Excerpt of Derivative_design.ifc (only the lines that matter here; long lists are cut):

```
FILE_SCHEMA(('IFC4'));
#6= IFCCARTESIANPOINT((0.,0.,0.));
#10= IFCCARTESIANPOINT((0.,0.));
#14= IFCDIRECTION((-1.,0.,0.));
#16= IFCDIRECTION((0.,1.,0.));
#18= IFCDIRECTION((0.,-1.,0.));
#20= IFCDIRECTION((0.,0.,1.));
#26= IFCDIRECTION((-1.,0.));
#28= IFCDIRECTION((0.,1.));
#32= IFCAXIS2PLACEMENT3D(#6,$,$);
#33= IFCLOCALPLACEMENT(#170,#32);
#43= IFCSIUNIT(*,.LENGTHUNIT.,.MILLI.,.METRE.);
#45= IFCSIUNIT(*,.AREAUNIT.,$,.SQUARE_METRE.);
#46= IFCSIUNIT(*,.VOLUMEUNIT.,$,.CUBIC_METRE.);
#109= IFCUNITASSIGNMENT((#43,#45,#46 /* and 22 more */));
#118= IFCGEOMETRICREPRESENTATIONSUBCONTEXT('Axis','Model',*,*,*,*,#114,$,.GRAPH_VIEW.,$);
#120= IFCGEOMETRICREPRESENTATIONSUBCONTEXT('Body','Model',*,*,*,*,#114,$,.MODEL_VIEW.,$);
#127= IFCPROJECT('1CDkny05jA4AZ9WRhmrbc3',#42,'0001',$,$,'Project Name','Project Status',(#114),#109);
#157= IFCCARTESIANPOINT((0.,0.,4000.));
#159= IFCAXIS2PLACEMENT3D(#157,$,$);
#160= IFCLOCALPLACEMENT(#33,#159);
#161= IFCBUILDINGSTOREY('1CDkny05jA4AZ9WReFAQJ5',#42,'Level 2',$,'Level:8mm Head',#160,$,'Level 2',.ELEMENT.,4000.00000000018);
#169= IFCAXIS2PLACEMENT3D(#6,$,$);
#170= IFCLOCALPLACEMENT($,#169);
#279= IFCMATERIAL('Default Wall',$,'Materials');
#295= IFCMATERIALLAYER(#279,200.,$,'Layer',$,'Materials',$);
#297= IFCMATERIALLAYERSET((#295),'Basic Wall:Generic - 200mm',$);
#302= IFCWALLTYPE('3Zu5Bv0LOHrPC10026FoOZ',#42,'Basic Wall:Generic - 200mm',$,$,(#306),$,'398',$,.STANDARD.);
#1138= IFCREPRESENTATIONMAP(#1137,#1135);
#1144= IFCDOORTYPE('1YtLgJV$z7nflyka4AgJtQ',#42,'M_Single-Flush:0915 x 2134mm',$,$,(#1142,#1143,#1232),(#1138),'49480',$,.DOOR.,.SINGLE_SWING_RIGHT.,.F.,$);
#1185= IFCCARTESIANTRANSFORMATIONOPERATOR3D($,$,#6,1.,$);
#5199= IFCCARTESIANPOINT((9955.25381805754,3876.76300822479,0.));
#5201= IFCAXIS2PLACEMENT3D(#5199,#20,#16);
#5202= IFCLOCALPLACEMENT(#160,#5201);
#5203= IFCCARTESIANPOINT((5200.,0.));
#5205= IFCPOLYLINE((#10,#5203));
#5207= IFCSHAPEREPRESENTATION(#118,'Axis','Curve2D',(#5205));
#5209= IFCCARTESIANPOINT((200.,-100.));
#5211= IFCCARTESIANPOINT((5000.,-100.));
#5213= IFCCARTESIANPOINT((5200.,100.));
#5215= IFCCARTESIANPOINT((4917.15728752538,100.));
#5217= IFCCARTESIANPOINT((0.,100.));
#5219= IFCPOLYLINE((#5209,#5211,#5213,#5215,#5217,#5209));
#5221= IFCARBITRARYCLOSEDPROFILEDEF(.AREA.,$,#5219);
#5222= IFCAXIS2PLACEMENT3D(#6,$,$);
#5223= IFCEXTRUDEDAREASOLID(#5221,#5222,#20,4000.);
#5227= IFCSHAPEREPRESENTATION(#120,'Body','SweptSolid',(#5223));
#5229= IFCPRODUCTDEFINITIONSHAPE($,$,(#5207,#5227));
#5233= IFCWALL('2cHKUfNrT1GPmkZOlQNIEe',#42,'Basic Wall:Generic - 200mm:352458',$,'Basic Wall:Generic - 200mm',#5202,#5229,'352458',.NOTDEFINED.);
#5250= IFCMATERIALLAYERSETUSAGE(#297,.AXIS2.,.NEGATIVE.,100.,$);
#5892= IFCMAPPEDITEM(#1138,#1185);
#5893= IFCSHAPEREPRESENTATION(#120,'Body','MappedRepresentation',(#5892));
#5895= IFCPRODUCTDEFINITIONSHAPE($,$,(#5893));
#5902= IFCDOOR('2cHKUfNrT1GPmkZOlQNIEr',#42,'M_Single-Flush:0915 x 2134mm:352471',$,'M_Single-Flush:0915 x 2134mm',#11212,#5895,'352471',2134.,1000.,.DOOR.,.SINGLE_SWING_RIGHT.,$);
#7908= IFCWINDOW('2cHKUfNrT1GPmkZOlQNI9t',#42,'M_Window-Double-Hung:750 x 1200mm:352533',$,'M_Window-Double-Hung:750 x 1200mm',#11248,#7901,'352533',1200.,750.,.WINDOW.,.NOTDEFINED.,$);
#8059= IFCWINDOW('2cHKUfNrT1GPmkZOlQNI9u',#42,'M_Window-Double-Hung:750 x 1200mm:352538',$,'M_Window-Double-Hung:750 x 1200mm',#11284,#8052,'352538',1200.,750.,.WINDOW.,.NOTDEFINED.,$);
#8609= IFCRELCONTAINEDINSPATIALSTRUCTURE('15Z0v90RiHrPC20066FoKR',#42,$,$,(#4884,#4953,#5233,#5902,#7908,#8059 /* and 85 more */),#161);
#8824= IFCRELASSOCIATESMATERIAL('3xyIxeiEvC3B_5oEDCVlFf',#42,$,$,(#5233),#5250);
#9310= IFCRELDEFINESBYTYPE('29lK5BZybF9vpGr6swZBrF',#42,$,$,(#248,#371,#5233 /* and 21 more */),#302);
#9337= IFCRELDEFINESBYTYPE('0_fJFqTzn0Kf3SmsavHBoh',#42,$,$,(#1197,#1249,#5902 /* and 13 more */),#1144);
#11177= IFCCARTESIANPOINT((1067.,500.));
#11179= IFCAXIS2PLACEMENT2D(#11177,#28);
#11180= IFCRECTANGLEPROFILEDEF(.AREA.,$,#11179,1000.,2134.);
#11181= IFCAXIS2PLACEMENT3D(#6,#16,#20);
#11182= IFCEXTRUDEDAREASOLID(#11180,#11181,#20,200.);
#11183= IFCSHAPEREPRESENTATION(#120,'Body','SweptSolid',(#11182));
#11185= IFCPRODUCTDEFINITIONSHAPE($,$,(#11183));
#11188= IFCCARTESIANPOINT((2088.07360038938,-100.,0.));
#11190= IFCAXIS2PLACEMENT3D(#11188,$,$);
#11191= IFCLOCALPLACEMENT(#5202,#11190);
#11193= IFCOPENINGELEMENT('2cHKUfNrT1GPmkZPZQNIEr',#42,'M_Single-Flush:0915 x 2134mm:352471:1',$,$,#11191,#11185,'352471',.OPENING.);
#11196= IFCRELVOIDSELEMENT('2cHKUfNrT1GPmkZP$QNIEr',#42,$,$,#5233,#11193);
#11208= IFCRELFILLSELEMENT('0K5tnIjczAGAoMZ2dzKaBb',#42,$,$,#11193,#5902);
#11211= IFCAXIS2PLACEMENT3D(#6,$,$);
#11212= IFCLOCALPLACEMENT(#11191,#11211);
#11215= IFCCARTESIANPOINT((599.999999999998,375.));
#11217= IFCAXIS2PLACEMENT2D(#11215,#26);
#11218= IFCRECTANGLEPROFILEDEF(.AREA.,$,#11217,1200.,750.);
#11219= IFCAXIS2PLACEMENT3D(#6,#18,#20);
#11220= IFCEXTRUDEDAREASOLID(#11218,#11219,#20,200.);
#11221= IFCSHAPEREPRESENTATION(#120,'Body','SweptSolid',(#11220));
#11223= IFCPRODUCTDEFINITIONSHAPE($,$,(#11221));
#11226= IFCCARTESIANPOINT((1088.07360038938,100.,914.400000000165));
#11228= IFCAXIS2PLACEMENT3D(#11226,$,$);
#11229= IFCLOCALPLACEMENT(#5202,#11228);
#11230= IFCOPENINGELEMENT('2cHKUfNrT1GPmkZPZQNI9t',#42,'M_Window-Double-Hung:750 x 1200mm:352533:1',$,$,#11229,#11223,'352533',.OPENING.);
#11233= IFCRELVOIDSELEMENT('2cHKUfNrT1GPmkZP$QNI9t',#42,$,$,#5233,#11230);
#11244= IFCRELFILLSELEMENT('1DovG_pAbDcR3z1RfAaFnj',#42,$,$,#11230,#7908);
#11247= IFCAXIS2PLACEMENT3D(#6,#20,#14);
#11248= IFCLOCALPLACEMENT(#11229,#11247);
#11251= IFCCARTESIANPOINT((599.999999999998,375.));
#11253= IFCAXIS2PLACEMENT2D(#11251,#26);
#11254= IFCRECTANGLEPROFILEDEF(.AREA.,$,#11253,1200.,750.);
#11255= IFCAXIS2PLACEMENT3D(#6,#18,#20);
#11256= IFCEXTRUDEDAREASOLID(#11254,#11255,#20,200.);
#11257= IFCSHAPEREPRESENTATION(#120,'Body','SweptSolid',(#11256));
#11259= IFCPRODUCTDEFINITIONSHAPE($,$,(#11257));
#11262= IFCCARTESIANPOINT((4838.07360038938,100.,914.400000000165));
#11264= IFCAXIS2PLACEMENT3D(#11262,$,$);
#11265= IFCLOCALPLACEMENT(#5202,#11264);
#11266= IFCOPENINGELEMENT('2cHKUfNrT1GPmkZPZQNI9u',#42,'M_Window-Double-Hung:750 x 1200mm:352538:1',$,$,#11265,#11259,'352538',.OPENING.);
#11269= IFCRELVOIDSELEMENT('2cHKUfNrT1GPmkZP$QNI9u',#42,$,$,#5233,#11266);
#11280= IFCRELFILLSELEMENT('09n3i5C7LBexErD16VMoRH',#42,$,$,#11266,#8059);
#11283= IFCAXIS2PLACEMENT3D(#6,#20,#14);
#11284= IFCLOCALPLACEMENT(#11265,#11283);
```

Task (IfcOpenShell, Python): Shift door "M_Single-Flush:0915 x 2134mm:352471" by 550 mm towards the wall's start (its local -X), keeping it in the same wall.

```python
import ifcopenshell
import ifcopenshell.api.geometry
import ifcopenshell.util.placement

model = ifcopenshell.open("Derivative_design.ifc")

door = model.by_id(5902)
opening = door.FillsVoids[0].RelatingOpeningElement
wall = opening.VoidsElements[0].RelatingBuildingElement

wall_matrix = ifcopenshell.util.placement.get_local_placement(wall.ObjectPlacement)
shift = wall_matrix[:3, 0] * -550.0
before = ifcopenshell.util.placement.get_local_placement(door.ObjectPlacement)[:3, 3].copy()

# The door is placed relative to its opening, so it follows when the opening moves.
matrix = ifcopenshell.util.placement.get_local_placement(opening.ObjectPlacement)
matrix[:3, 3] += shift
ifcopenshell.api.geometry.edit_object_placement(
    model, product=opening, matrix=matrix, is_si=False, should_transform_children=True
)

after = ifcopenshell.util.placement.get_local_placement(door.ObjectPlacement)[:3, 3]
print("door moved by", (after - before).round(3) + 0.0)

model.write("Derivative_design_v2.ifc")
```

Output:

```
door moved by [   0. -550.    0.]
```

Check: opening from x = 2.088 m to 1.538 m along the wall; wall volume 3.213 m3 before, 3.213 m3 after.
